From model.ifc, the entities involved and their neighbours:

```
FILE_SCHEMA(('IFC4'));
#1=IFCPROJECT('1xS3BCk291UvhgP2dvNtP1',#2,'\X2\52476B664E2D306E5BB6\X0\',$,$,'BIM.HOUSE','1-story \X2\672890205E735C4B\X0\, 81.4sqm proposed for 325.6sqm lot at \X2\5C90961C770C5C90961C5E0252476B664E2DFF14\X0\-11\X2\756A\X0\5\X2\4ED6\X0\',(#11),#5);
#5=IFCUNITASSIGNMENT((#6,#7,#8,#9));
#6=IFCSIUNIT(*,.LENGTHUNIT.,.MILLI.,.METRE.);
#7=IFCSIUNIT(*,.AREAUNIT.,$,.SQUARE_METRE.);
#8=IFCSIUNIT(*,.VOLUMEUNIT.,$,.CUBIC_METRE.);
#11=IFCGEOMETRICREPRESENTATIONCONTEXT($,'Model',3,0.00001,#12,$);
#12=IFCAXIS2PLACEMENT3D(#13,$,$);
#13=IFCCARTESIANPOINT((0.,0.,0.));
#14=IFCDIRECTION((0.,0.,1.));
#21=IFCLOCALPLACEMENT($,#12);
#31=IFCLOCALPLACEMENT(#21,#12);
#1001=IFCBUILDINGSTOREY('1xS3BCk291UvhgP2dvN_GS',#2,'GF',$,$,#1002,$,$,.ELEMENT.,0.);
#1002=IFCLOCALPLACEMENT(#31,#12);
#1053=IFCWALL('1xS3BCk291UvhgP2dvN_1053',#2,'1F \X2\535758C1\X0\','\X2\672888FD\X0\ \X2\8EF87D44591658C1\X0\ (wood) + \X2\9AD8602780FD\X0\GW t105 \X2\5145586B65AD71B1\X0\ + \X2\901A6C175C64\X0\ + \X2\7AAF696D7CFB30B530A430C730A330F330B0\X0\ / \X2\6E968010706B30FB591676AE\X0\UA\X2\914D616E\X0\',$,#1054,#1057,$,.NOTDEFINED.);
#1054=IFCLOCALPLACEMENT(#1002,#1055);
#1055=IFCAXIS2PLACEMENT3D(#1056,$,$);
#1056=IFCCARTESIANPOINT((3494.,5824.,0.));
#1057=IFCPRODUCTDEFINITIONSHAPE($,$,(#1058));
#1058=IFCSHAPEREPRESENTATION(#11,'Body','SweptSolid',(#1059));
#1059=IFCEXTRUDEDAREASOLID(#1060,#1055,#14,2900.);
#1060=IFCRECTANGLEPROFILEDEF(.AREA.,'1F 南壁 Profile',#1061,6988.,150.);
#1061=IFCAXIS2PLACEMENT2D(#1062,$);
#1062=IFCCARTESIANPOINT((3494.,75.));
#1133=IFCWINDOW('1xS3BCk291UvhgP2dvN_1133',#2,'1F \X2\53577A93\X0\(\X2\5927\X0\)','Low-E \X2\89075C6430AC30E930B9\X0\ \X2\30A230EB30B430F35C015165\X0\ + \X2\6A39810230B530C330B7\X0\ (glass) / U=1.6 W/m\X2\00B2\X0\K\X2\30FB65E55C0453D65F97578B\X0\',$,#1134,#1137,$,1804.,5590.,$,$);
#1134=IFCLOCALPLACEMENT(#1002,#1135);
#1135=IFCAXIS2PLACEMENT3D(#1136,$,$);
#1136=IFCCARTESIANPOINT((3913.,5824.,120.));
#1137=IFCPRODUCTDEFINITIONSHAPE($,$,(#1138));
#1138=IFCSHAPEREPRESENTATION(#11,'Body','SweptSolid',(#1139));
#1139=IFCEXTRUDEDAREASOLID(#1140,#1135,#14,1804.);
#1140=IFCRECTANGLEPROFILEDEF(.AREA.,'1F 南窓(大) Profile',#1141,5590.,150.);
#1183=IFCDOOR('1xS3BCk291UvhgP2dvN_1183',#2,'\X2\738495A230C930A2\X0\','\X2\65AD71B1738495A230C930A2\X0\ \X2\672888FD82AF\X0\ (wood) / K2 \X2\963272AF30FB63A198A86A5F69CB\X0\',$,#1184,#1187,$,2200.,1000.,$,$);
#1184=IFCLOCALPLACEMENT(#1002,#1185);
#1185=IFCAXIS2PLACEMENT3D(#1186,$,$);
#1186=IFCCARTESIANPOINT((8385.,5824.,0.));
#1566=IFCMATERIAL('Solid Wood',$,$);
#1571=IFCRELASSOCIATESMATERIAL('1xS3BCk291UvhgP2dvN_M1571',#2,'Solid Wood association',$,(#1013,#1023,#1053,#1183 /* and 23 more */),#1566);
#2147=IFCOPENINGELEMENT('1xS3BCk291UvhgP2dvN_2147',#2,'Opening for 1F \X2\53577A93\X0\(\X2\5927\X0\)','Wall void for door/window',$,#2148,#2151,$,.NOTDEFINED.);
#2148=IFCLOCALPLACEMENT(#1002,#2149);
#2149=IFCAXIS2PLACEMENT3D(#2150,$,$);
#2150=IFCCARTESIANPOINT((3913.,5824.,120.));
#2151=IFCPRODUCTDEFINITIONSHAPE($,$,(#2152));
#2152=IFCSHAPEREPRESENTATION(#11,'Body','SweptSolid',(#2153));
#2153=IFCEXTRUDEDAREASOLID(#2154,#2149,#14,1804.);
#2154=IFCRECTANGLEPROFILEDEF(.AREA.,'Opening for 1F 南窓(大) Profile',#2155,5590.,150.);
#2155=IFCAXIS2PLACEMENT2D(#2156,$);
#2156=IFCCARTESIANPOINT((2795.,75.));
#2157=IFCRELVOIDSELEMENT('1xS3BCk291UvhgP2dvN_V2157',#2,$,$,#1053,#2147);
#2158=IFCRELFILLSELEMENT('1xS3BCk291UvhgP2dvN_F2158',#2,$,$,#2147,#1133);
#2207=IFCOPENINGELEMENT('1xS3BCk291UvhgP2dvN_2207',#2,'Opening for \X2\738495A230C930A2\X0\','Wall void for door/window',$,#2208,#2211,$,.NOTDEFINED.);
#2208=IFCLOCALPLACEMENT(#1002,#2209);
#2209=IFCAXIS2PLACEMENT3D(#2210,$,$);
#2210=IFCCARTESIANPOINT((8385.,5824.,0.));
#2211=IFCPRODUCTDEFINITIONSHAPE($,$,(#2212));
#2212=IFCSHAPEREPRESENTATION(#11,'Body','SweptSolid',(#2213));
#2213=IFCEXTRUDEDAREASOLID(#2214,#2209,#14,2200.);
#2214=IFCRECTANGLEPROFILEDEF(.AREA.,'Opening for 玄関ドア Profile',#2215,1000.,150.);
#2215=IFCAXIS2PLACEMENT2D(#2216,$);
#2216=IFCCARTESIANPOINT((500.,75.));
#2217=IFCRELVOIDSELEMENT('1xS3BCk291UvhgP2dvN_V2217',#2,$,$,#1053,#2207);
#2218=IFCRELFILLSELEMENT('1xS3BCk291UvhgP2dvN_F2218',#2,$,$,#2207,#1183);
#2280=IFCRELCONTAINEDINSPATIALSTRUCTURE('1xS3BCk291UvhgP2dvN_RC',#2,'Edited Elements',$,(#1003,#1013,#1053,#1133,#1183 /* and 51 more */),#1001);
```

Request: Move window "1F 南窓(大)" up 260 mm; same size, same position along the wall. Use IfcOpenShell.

```python
import numpy as np
import ifcopenshell
import ifcopenshell.api.geometry
import ifcopenshell.util.placement
import ifcopenshell.util.unit

model = ifcopenshell.open("model.ifc")
unit_scale = ifcopenshell.util.unit.calculate_unit_scale(model)

window = model.by_guid("1xS3BCk291UvhgP2dvN_1133")
opening = window.FillsVoids[0].RelatingOpeningElement
dz = 0.26 / unit_scale

shift = np.array([0.0, 0.0, dz])
# The window is not placed relative to its opening, so move both.
for product in (opening, window):
    matrix = ifcopenshell.util.placement.get_local_placement(product.ObjectPlacement)
    matrix[:3, 3] += shift
    ifcopenshell.api.geometry.edit_object_placement(model, product=product, matrix=matrix, is_si=False)

print(f"moved by {dz * unit_scale:+.3f} m")

model.write("model_rev.ifc")
```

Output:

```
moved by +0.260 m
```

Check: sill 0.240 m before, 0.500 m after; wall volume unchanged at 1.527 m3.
